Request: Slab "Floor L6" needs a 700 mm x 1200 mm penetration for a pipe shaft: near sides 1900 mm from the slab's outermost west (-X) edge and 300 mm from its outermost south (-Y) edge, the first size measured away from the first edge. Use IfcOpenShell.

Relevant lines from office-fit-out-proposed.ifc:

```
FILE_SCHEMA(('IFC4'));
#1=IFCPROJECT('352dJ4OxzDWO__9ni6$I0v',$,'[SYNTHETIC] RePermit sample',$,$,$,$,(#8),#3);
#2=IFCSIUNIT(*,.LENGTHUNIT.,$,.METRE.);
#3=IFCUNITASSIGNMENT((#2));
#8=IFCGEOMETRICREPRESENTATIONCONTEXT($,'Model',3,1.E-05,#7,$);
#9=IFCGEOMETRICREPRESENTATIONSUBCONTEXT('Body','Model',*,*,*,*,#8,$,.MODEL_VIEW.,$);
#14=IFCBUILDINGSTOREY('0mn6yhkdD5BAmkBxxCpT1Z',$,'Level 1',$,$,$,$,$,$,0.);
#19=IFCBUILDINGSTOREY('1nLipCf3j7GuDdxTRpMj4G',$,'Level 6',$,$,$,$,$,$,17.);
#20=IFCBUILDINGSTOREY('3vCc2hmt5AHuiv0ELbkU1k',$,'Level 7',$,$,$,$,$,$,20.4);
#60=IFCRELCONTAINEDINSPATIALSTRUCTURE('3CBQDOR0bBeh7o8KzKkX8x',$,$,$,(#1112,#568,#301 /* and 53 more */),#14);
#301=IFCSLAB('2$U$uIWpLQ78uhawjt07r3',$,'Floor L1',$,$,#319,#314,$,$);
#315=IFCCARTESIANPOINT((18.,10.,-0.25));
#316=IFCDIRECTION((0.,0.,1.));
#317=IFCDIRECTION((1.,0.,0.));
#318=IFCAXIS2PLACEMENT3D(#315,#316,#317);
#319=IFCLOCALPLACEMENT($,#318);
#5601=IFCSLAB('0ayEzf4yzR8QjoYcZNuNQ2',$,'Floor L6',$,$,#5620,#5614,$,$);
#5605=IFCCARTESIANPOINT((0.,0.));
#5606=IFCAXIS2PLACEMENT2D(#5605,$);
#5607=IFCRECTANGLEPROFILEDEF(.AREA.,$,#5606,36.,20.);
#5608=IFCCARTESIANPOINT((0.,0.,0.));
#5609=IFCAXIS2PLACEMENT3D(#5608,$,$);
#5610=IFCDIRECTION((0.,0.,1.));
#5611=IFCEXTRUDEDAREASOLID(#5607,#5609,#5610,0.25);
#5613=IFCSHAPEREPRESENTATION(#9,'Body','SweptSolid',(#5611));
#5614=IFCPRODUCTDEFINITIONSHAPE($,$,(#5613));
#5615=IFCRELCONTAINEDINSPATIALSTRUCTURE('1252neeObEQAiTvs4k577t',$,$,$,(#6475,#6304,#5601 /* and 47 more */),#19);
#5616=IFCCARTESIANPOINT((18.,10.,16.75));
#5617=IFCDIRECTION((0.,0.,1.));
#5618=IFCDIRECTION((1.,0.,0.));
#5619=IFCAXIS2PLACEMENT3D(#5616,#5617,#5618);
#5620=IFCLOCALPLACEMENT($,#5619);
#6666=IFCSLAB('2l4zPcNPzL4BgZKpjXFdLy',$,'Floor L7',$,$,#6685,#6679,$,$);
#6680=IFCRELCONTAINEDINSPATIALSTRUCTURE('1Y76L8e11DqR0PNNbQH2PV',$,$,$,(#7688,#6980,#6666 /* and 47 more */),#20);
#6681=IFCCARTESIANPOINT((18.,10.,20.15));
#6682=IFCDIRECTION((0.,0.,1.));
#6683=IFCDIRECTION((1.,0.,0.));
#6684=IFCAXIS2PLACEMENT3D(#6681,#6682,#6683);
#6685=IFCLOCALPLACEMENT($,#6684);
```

```python
import numpy as np
import ifcopenshell
import ifcopenshell.api.feature
import ifcopenshell.api.geometry
import ifcopenshell.api.root
import ifcopenshell.geom
import ifcopenshell.util.placement
import ifcopenshell.util.representation
import ifcopenshell.util.shape
import ifcopenshell.util.unit

model = ifcopenshell.open("office-fit-out-proposed.ifc")
unit_scale = ifcopenshell.util.unit.calculate_unit_scale(model)
settings = ifcopenshell.geom.settings()


def volume(element):
    """Net volume in cubic metres, openings subtracted."""
    shape = ifcopenshell.geom.create_shape(settings, element)
    return ifcopenshell.util.shape.get_volume(shape.geometry)


slab = model.by_guid("0ayEzf4yzR8QjoYcZNuNQ2")
before = volume(slab)

# Extent in the slab's own axes, in metres. The edges named are its -X and -Y sides.
slab_shape = ifcopenshell.geom.create_shape(settings, slab)
vertices = ifcopenshell.util.shape.get_vertices(slab_shape.geometry)
x_min, y_min, bottom = vertices.min(axis=0)
top = vertices[:, 2].max()

opening = ifcopenshell.api.root.create_entity(model, ifc_class="IfcOpeningElement", name="Pipe shaft opening", predefined_type="OPENING")
context = ifcopenshell.util.representation.get_context(model, "Model", "Body", "MODEL_VIEW")
width, depth = 0.7, 1.2
outline = [(0.0, 0.0), (width, 0.0), (width, depth), (0.0, depth), (0.0, 0.0)]
# Overshoot both faces by 50 mm so the cut is clean.
shape = ifcopenshell.api.geometry.add_slab_representation(
    model, context=context, depth=top - bottom + 0.1, polyline=outline
)
ifcopenshell.api.geometry.assign_representation(model, product=opening, representation=shape)

matrix = ifcopenshell.util.placement.get_local_placement(slab.ObjectPlacement)
matrix[:, 3] = matrix @ np.append(np.array([x_min + 1.9, y_min + 0.3, bottom - 0.05]) / unit_scale, 1.0)
ifcopenshell.api.geometry.edit_object_placement(model, product=opening, matrix=matrix, is_si=False)
ifcopenshell.api.feature.add_feature(model, feature=opening, element=slab)

after = volume(slab)

print(f"slab volume {before:.3f} -> {after:.3f} m3")

model.write("office-fit-out-proposed-out.ifc")
```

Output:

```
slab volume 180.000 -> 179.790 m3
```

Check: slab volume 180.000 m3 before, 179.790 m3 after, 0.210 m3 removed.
